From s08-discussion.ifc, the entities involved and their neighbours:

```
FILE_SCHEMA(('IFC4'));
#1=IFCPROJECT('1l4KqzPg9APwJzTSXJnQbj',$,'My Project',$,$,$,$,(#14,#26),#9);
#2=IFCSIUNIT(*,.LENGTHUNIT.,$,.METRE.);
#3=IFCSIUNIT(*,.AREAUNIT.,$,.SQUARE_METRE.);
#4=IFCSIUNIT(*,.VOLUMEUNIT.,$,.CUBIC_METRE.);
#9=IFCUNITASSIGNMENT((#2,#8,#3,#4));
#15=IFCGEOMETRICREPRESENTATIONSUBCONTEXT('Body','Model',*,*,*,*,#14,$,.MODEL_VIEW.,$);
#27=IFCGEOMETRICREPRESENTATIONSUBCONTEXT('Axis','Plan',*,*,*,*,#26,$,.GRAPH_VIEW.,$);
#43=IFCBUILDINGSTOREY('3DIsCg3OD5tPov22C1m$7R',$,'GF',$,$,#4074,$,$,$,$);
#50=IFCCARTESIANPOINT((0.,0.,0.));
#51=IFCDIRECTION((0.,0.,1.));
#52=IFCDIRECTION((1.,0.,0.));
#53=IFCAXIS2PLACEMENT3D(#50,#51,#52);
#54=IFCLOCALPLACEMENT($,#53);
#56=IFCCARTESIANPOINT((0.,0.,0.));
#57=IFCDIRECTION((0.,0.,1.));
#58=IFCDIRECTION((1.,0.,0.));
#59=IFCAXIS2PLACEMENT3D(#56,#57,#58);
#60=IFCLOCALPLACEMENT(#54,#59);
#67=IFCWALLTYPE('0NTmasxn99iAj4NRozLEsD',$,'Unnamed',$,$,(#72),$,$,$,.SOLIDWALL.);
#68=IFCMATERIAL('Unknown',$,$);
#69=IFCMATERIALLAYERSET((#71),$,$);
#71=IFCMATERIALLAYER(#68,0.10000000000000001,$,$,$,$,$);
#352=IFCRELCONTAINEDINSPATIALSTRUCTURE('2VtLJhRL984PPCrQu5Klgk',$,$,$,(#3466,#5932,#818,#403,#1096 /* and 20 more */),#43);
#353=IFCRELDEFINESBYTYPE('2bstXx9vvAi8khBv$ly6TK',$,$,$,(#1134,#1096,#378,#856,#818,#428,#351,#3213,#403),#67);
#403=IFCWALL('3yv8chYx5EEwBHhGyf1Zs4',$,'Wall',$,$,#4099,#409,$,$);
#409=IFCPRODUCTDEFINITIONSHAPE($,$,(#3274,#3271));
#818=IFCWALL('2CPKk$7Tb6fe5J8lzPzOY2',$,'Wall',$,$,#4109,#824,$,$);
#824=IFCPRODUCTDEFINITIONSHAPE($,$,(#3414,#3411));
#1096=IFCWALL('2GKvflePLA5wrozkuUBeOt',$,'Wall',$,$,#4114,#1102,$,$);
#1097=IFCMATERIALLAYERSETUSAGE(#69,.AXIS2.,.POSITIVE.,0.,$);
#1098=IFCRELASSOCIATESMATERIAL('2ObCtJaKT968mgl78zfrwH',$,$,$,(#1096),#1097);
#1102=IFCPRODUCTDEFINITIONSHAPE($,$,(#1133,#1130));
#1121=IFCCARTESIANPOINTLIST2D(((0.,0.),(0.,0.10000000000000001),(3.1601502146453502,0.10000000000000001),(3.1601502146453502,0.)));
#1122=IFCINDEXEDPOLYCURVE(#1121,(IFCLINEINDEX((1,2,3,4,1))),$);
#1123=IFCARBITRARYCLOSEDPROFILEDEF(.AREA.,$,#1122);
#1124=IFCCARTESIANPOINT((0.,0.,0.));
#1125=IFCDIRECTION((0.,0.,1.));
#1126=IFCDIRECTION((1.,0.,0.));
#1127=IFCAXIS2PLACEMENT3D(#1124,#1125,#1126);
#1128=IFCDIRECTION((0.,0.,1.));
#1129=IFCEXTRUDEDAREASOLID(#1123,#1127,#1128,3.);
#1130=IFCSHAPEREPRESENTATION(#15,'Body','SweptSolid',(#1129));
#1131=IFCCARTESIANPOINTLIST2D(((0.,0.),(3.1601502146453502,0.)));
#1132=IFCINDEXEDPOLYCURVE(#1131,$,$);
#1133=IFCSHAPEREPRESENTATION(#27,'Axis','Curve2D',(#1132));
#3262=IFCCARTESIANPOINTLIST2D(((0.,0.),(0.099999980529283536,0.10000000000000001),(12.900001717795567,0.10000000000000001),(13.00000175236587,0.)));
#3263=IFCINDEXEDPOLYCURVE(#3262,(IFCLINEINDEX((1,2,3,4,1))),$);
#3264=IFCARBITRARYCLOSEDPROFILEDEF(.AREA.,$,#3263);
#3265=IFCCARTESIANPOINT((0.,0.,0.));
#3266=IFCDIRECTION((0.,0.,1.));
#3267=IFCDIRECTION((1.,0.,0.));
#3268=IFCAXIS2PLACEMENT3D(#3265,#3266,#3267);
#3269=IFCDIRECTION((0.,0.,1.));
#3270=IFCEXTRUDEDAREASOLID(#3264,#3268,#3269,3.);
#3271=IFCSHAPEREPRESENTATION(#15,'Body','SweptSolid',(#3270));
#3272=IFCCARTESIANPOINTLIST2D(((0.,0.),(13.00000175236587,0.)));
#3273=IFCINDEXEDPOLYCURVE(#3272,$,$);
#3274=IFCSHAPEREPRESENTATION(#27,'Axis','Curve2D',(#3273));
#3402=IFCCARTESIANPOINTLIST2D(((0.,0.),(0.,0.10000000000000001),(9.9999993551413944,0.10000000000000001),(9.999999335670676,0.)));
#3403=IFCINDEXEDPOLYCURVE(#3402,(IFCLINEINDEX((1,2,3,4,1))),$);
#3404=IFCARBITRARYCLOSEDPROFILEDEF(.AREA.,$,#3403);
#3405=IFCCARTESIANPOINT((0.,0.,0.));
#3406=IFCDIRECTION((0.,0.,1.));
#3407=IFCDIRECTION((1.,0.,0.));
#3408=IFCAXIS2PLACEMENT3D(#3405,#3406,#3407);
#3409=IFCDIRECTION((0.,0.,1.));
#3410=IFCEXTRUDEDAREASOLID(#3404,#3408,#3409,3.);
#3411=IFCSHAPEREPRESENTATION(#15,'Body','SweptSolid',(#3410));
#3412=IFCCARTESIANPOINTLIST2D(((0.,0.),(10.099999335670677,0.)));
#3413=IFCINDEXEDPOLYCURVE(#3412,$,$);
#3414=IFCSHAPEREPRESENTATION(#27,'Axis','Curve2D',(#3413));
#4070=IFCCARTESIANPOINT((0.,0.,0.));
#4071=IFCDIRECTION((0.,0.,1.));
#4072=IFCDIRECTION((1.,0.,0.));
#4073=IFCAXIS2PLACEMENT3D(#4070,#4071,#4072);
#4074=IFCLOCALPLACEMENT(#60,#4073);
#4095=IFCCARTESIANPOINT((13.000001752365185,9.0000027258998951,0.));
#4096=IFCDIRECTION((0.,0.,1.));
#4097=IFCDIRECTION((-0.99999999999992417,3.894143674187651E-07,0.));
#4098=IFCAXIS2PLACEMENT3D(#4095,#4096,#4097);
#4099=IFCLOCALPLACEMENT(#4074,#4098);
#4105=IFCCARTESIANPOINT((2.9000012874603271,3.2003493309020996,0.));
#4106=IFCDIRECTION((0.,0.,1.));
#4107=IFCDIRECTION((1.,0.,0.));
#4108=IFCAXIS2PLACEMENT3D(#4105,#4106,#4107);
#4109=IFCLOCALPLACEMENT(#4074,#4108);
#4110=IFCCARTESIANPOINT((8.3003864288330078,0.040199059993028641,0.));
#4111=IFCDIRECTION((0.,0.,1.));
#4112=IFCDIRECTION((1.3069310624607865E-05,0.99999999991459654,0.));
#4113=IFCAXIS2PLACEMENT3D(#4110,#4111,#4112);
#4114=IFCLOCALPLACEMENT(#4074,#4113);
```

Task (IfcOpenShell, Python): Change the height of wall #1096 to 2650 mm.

```python
import ifcopenshell
import ifcopenshell.geom
import ifcopenshell.util.representation
import ifcopenshell.util.shape
import ifcopenshell.util.unit

model = ifcopenshell.open("s08-discussion.ifc")
unit_scale = ifcopenshell.util.unit.calculate_unit_scale(model)
settings = ifcopenshell.geom.settings()


def volume(element):
    """Net volume in cubic metres, openings subtracted."""
    shape = ifcopenshell.geom.create_shape(settings, element)
    return ifcopenshell.util.shape.get_volume(shape.geometry)


wall = model.by_guid("2GKvflePLA5wrozkuUBeOt")
before = volume(wall)

body = ifcopenshell.util.representation.get_representation(wall, "Model", "Body")
solid = body.Items[0]
old_height = solid.Depth
solid.Depth = 2.65 / unit_scale
after = volume(wall)

print(f"height {old_height:g} -> {solid.Depth:g}, volume {before:.3f} -> {after:.3f} m3")

model.write("s08-discussion_updated.ifc")
```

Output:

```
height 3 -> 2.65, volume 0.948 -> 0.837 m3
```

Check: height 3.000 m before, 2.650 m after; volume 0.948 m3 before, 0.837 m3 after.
